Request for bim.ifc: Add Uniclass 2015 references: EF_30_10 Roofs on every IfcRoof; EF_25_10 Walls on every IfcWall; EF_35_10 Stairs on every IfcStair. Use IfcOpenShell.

First a look at what the model holds.

```python
import ifcopenshell

model = ifcopenshell.open("bim.ifc")
print(model.schema)
print("classifications:", [c.Name for c in model.by_type("IfcClassification")])
for ifc_class in ("IfcDoor", "IfcRoof", "IfcStair", "IfcWall", "IfcWindow"):
    print(ifc_class, len(model.by_type(ifc_class)))
```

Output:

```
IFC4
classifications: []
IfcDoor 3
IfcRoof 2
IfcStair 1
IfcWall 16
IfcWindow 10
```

```python
import ifcopenshell
import ifcopenshell.api.classification

model = ifcopenshell.open("bim.ifc")

system = ifcopenshell.api.classification.add_classification(model, classification="Uniclass 2015")

codes = {
    "IfcRoof": ("EF_30_10", "Roofs"),
    "IfcWall": ("EF_25_10", "Walls"),
    "IfcStair": ("EF_35_10", "Stairs"),
}
for ifc_class, (code, name) in codes.items():
    products = model.by_type(ifc_class)
    ifcopenshell.api.classification.add_reference(
        model, products=products, classification=system, identification=code, name=name
    )
    print(code, len(products))

model.write("bim_updated.ifc")
```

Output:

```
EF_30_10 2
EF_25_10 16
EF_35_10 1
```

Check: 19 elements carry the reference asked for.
